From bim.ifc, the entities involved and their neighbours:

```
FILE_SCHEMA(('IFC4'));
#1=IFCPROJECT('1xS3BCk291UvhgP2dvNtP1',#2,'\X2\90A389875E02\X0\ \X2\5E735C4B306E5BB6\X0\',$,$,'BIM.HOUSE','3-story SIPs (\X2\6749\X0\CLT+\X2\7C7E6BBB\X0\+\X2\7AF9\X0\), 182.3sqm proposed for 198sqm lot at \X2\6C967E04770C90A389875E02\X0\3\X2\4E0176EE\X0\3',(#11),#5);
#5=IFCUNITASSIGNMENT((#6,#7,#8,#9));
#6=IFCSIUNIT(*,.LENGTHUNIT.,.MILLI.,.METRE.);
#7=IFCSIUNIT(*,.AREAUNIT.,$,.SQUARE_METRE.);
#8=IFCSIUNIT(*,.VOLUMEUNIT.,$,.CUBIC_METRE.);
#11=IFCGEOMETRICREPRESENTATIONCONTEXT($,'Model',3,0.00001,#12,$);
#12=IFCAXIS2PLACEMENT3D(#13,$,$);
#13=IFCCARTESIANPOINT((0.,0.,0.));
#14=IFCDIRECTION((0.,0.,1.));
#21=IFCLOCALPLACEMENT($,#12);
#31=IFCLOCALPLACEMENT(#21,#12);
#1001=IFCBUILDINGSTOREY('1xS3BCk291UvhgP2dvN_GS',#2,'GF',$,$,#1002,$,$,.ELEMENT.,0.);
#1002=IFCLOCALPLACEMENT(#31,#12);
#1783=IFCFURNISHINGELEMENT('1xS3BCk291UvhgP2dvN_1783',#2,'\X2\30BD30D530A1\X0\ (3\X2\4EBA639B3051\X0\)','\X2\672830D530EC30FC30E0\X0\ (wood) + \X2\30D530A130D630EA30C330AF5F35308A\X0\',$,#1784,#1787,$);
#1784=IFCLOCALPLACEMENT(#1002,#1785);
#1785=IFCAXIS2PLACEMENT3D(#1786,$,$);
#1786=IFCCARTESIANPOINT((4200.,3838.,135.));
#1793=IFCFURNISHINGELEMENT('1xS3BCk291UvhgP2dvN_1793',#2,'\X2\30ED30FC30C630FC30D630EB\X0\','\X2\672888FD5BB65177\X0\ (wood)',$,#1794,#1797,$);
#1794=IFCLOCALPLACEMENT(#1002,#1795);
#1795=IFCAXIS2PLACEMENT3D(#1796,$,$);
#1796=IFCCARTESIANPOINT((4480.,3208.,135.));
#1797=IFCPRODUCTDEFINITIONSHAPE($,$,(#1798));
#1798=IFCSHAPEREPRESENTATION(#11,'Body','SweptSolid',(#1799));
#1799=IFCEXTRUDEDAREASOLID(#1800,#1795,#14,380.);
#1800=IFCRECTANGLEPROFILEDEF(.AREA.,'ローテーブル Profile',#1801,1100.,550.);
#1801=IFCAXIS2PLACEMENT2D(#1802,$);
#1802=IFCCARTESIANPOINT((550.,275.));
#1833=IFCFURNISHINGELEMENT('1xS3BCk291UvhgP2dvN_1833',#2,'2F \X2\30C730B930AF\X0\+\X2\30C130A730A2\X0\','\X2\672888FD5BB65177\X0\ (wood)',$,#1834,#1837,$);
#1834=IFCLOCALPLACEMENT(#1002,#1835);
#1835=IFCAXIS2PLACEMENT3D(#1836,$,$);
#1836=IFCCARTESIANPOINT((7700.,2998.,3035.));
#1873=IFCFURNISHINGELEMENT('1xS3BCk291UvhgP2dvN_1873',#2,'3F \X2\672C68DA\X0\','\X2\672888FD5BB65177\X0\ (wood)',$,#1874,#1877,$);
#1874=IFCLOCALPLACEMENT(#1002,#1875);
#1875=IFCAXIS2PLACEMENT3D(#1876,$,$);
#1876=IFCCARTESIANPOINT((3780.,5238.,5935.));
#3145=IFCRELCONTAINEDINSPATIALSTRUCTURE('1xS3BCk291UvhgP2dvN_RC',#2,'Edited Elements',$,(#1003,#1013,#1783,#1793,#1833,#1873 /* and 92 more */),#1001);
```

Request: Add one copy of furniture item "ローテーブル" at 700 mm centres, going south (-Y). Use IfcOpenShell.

```python
import numpy as np
import ifcopenshell
import ifcopenshell.api.geometry
import ifcopenshell.api.root
import ifcopenshell.util.element
import ifcopenshell.util.placement
import ifcopenshell.util.unit

model = ifcopenshell.open("bim.ifc")
unit_scale = ifcopenshell.util.unit.calculate_unit_scale(model)


def reuse_history(source, copy):
    """copy_class also copies each property set's owner history, people and application; keep the originals."""
    for rel in copy.IsDefinedBy:
        if rel.is_a("IfcRelDefinesByProperties") and (history := rel.RelatingPropertyDefinition.OwnerHistory):
            rel.RelatingPropertyDefinition.OwnerHistory = source.OwnerHistory
            ifcopenshell.util.element.remove_deep2(model, history)


source = model.by_guid("1xS3BCk291UvhgP2dvN_1793")
base = ifcopenshell.util.placement.get_local_placement(source.ObjectPlacement)
step = np.array([0.0, -1.0, 0.0]) * 0.7 / unit_scale

for i in range(1, 2):
    copy = ifcopenshell.api.root.copy_class(model, product=source)
    copy.Representation = ifcopenshell.util.element.copy_deep(
        model, source.Representation, exclude=["IfcGeometricRepresentationContext", "IfcRepresentationMap"]
    )
    reuse_history(source, copy)
    matrix = base.copy()
    matrix[:3, 3] += i * step
    print("added at", matrix[:3, 3].round(3) + 0.0)
    ifcopenshell.api.geometry.edit_object_placement(model, product=copy, matrix=matrix, is_si=False)

model.write("bim_edited.ifc")
```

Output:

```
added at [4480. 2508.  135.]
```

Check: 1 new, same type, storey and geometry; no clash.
